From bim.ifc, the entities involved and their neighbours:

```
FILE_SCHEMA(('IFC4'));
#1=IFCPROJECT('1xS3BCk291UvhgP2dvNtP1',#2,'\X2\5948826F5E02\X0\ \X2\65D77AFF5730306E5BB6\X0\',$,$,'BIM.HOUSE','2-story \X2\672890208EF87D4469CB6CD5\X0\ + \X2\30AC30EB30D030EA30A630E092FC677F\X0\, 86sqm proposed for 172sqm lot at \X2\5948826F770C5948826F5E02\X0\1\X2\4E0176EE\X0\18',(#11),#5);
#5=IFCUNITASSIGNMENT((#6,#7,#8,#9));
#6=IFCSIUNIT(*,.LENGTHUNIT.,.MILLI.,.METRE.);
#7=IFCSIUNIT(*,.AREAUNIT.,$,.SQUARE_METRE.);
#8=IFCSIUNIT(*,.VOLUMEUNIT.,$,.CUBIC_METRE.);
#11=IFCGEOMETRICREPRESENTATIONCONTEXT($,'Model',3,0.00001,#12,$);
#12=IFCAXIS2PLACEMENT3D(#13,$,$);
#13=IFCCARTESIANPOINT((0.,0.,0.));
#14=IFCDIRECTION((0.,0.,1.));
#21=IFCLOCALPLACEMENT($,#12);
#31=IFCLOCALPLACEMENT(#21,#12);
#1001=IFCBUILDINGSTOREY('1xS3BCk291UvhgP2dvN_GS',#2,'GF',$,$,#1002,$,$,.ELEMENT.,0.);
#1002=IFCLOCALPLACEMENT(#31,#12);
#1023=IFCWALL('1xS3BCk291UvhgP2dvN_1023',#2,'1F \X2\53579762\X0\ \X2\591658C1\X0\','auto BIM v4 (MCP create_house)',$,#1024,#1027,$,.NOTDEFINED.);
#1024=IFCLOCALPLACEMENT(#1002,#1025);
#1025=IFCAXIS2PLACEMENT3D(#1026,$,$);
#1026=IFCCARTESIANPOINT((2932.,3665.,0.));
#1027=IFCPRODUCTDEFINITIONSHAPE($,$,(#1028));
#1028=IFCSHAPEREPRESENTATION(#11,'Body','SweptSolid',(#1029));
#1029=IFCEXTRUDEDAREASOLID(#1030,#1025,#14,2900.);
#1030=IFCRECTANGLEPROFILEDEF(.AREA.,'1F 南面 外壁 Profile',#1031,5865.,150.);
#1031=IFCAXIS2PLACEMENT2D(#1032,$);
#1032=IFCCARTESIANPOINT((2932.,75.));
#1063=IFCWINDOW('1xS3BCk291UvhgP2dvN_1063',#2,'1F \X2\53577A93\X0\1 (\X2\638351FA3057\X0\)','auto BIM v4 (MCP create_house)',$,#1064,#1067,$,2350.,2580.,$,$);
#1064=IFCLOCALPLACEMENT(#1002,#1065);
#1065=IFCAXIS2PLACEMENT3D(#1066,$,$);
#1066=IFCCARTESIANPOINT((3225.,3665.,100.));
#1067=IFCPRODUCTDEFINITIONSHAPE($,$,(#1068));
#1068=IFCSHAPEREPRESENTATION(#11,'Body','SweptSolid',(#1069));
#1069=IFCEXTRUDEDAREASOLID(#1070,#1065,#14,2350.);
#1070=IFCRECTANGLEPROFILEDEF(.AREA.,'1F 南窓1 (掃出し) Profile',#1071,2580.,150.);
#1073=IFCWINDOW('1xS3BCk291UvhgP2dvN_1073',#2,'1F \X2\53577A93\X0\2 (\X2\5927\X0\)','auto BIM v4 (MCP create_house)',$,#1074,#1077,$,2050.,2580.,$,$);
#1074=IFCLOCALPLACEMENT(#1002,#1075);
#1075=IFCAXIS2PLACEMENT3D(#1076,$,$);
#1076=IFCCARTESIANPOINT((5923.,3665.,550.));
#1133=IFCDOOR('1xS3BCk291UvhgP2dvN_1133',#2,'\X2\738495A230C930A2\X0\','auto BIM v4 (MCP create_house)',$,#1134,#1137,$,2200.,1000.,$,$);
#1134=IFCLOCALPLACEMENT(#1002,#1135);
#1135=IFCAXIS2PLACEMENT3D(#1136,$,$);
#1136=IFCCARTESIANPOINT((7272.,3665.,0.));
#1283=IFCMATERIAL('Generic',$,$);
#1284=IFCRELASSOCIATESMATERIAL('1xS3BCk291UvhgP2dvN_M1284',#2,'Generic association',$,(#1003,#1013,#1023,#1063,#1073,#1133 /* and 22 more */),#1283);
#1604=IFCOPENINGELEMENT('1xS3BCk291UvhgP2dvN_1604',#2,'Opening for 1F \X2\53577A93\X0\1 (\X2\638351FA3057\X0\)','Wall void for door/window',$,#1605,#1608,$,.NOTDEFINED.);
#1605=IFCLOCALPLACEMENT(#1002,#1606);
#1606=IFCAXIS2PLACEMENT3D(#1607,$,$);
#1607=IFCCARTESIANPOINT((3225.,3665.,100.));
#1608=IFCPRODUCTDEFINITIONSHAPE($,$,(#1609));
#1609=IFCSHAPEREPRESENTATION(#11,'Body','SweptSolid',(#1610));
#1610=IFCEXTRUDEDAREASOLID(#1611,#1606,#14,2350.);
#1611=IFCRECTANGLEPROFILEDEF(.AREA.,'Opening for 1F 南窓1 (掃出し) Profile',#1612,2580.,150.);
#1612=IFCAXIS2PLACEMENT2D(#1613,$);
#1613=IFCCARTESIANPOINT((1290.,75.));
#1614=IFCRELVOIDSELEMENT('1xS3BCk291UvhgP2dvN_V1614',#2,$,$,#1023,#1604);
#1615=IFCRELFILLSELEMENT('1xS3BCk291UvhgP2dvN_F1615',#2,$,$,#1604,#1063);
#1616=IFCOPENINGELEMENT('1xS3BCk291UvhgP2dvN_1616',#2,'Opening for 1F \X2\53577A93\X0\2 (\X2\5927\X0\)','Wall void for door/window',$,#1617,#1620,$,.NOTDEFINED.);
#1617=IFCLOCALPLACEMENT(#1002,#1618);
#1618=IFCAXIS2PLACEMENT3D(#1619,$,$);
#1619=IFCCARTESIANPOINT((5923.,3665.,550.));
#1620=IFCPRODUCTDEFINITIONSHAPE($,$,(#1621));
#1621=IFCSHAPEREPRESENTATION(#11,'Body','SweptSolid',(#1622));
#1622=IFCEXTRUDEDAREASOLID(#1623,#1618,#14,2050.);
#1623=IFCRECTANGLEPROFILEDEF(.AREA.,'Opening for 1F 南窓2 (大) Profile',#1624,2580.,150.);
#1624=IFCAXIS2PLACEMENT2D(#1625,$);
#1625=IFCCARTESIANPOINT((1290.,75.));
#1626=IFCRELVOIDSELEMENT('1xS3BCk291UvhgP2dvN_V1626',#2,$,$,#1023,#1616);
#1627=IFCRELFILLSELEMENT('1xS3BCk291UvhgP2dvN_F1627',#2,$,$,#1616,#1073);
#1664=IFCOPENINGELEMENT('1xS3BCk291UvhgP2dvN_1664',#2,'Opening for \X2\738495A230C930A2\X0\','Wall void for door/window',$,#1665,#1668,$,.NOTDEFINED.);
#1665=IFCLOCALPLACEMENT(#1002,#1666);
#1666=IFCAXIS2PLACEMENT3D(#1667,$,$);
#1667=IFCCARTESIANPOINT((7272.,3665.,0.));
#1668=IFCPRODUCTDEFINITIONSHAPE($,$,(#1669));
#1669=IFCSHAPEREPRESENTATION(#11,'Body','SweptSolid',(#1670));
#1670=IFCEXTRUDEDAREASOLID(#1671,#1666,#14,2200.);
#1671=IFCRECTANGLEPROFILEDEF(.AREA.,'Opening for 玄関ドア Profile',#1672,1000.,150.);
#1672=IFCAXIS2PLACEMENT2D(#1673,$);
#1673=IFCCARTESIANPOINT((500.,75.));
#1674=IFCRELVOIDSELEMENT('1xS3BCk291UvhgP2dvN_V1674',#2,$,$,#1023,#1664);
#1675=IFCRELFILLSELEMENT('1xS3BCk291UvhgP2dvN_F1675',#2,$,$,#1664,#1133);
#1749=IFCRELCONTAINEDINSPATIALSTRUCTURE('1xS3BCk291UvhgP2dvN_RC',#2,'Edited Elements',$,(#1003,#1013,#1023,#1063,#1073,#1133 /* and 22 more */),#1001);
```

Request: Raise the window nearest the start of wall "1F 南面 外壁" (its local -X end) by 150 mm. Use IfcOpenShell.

```python
import numpy as np
import ifcopenshell
import ifcopenshell.api.geometry
import ifcopenshell.util.placement
import ifcopenshell.util.unit

model = ifcopenshell.open("bim.ifc")
unit_scale = ifcopenshell.util.unit.calculate_unit_scale(model)

window = model.by_guid("1xS3BCk291UvhgP2dvN_1063")
opening = window.FillsVoids[0].RelatingOpeningElement
dz = 0.15 / unit_scale

shift = np.array([0.0, 0.0, dz])
# The window is not placed relative to its opening, so move both.
for product in (opening, window):
    matrix = ifcopenshell.util.placement.get_local_placement(product.ObjectPlacement)
    matrix[:3, 3] += shift
    ifcopenshell.api.geometry.edit_object_placement(model, product=product, matrix=matrix, is_si=False)

print(f"moved by {dz * unit_scale:+.3f} m")

model.write("bim_edited.ifc")
```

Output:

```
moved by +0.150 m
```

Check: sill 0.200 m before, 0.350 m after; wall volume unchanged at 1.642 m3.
